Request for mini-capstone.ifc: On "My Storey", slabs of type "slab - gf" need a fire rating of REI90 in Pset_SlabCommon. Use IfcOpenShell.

First a look at what the model holds.

```python
import ifcopenshell
import ifcopenshell.util.element

model = ifcopenshell.open("mini-capstone.ifc")
print(model.schema)
storey = next(s for s in model.by_type("IfcBuildingStorey") if s.Name == "My Storey")
slabs = [e for e in ifcopenshell.util.element.get_decomposition(storey) if e.is_a("IfcSlab")]
seen = {}
for e in slabs:
    element_type = ifcopenshell.util.element.get_type(e)
    key = (element_type.Name if element_type != e and element_type else None, ifcopenshell.util.element.get_pset(e, "Pset_SlabCommon", "FireRating"))
    seen[key] = seen.get(key, 0) + 1
for (name, value), count in sorted(seen.items(), key=str):
    print(count, "x", name, "|", value)
```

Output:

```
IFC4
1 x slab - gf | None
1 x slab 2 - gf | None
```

```python
import ifcopenshell
import ifcopenshell.api.pset
import ifcopenshell.util.element

model = ifcopenshell.open("mini-capstone.ifc")

storey = next(s for s in model.by_type("IfcBuildingStorey") if s.Name == "My Storey")
slabs = [e for e in ifcopenshell.util.element.get_decomposition(storey) if e.is_a("IfcSlab")]

count = 0
for e in slabs:
    element_type = ifcopenshell.util.element.get_type(e)
    if element_type in (None, e) or element_type.Name != "slab - gf":
        continue
    # add_pset returns the element's existing set when there is one.
    pset = ifcopenshell.api.pset.add_pset(model, product=e, name="Pset_SlabCommon")
    ifcopenshell.api.pset.edit_pset(model, pset=pset, properties={"FireRating": "REI90"})
    count += 1

print(count, "slabs updated")

model.write("mini-capstone_updated.ifc")
```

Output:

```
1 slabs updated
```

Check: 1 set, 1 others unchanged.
